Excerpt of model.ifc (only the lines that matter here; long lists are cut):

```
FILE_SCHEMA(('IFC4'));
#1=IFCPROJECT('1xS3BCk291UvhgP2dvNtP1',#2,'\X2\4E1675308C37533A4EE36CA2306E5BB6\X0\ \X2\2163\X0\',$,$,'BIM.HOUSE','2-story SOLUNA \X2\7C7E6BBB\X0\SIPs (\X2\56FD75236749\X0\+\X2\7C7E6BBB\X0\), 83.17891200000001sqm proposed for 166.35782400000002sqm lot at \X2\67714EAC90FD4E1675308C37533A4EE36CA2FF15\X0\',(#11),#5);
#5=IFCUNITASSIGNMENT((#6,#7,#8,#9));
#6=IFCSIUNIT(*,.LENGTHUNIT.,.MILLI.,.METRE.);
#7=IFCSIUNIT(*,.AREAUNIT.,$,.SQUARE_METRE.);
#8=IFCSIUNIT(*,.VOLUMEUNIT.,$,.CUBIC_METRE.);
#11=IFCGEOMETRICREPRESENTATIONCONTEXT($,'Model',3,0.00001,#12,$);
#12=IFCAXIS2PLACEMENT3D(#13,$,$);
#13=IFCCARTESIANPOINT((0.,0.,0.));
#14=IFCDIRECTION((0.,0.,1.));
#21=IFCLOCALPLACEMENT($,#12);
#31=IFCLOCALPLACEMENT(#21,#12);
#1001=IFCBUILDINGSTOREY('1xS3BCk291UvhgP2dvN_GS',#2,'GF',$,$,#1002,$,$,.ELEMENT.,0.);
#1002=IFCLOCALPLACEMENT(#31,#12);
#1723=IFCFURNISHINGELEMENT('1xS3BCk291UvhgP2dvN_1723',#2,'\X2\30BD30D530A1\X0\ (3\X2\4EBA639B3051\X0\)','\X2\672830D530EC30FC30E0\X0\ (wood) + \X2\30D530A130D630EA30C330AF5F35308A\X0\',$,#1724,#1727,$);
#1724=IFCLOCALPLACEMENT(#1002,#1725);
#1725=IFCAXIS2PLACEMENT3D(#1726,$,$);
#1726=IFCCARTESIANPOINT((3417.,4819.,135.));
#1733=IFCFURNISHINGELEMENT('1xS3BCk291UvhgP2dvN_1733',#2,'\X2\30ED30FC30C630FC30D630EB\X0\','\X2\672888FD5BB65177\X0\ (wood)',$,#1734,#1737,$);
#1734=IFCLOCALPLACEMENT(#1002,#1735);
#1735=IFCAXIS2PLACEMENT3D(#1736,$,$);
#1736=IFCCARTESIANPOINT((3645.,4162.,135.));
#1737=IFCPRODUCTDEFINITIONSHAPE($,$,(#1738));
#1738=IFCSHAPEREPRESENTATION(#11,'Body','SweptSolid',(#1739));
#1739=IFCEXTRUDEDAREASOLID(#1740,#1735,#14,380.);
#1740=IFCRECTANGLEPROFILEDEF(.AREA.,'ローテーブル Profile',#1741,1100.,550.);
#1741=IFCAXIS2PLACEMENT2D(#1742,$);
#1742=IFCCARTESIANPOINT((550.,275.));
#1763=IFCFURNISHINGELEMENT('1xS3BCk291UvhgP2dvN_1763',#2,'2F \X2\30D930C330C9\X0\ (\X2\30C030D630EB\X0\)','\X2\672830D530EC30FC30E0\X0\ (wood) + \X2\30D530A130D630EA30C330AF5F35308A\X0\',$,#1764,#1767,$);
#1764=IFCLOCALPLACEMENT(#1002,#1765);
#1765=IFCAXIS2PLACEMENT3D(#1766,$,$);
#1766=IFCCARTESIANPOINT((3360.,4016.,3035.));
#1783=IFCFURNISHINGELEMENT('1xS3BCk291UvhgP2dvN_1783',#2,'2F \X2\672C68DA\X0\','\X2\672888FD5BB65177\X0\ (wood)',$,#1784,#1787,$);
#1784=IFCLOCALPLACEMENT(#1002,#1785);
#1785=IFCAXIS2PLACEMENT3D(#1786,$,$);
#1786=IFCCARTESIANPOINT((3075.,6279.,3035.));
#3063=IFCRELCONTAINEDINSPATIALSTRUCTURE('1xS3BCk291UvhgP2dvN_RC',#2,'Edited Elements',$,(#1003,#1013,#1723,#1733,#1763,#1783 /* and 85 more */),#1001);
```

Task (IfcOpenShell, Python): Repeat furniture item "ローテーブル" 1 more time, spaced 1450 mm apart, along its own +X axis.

```python
import ifcopenshell
import ifcopenshell.api.geometry
import ifcopenshell.api.root
import ifcopenshell.util.element
import ifcopenshell.util.placement
import ifcopenshell.util.unit

model = ifcopenshell.open("model.ifc")
unit_scale = ifcopenshell.util.unit.calculate_unit_scale(model)


def reuse_history(source, copy):
    """copy_class also copies each property set's owner history, people and application; keep the originals."""
    for rel in copy.IsDefinedBy:
        if rel.is_a("IfcRelDefinesByProperties") and (history := rel.RelatingPropertyDefinition.OwnerHistory):
            rel.RelatingPropertyDefinition.OwnerHistory = source.OwnerHistory
            ifcopenshell.util.element.remove_deep2(model, history)


source = model.by_guid("1xS3BCk291UvhgP2dvN_1733")
base = ifcopenshell.util.placement.get_local_placement(source.ObjectPlacement)
step = base[:3, 0] * 1.45 / unit_scale

for i in range(1, 2):
    copy = ifcopenshell.api.root.copy_class(model, product=source)
    copy.Representation = ifcopenshell.util.element.copy_deep(
        model, source.Representation, exclude=["IfcGeometricRepresentationContext", "IfcRepresentationMap"]
    )
    reuse_history(source, copy)
    matrix = base.copy()
    matrix[:3, 3] += i * step
    print("added at", matrix[:3, 3].round(3) + 0.0)
    ifcopenshell.api.geometry.edit_object_placement(model, product=copy, matrix=matrix, is_si=False)

model.write("model_v2.ifc")
```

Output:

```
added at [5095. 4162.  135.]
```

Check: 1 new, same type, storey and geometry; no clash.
